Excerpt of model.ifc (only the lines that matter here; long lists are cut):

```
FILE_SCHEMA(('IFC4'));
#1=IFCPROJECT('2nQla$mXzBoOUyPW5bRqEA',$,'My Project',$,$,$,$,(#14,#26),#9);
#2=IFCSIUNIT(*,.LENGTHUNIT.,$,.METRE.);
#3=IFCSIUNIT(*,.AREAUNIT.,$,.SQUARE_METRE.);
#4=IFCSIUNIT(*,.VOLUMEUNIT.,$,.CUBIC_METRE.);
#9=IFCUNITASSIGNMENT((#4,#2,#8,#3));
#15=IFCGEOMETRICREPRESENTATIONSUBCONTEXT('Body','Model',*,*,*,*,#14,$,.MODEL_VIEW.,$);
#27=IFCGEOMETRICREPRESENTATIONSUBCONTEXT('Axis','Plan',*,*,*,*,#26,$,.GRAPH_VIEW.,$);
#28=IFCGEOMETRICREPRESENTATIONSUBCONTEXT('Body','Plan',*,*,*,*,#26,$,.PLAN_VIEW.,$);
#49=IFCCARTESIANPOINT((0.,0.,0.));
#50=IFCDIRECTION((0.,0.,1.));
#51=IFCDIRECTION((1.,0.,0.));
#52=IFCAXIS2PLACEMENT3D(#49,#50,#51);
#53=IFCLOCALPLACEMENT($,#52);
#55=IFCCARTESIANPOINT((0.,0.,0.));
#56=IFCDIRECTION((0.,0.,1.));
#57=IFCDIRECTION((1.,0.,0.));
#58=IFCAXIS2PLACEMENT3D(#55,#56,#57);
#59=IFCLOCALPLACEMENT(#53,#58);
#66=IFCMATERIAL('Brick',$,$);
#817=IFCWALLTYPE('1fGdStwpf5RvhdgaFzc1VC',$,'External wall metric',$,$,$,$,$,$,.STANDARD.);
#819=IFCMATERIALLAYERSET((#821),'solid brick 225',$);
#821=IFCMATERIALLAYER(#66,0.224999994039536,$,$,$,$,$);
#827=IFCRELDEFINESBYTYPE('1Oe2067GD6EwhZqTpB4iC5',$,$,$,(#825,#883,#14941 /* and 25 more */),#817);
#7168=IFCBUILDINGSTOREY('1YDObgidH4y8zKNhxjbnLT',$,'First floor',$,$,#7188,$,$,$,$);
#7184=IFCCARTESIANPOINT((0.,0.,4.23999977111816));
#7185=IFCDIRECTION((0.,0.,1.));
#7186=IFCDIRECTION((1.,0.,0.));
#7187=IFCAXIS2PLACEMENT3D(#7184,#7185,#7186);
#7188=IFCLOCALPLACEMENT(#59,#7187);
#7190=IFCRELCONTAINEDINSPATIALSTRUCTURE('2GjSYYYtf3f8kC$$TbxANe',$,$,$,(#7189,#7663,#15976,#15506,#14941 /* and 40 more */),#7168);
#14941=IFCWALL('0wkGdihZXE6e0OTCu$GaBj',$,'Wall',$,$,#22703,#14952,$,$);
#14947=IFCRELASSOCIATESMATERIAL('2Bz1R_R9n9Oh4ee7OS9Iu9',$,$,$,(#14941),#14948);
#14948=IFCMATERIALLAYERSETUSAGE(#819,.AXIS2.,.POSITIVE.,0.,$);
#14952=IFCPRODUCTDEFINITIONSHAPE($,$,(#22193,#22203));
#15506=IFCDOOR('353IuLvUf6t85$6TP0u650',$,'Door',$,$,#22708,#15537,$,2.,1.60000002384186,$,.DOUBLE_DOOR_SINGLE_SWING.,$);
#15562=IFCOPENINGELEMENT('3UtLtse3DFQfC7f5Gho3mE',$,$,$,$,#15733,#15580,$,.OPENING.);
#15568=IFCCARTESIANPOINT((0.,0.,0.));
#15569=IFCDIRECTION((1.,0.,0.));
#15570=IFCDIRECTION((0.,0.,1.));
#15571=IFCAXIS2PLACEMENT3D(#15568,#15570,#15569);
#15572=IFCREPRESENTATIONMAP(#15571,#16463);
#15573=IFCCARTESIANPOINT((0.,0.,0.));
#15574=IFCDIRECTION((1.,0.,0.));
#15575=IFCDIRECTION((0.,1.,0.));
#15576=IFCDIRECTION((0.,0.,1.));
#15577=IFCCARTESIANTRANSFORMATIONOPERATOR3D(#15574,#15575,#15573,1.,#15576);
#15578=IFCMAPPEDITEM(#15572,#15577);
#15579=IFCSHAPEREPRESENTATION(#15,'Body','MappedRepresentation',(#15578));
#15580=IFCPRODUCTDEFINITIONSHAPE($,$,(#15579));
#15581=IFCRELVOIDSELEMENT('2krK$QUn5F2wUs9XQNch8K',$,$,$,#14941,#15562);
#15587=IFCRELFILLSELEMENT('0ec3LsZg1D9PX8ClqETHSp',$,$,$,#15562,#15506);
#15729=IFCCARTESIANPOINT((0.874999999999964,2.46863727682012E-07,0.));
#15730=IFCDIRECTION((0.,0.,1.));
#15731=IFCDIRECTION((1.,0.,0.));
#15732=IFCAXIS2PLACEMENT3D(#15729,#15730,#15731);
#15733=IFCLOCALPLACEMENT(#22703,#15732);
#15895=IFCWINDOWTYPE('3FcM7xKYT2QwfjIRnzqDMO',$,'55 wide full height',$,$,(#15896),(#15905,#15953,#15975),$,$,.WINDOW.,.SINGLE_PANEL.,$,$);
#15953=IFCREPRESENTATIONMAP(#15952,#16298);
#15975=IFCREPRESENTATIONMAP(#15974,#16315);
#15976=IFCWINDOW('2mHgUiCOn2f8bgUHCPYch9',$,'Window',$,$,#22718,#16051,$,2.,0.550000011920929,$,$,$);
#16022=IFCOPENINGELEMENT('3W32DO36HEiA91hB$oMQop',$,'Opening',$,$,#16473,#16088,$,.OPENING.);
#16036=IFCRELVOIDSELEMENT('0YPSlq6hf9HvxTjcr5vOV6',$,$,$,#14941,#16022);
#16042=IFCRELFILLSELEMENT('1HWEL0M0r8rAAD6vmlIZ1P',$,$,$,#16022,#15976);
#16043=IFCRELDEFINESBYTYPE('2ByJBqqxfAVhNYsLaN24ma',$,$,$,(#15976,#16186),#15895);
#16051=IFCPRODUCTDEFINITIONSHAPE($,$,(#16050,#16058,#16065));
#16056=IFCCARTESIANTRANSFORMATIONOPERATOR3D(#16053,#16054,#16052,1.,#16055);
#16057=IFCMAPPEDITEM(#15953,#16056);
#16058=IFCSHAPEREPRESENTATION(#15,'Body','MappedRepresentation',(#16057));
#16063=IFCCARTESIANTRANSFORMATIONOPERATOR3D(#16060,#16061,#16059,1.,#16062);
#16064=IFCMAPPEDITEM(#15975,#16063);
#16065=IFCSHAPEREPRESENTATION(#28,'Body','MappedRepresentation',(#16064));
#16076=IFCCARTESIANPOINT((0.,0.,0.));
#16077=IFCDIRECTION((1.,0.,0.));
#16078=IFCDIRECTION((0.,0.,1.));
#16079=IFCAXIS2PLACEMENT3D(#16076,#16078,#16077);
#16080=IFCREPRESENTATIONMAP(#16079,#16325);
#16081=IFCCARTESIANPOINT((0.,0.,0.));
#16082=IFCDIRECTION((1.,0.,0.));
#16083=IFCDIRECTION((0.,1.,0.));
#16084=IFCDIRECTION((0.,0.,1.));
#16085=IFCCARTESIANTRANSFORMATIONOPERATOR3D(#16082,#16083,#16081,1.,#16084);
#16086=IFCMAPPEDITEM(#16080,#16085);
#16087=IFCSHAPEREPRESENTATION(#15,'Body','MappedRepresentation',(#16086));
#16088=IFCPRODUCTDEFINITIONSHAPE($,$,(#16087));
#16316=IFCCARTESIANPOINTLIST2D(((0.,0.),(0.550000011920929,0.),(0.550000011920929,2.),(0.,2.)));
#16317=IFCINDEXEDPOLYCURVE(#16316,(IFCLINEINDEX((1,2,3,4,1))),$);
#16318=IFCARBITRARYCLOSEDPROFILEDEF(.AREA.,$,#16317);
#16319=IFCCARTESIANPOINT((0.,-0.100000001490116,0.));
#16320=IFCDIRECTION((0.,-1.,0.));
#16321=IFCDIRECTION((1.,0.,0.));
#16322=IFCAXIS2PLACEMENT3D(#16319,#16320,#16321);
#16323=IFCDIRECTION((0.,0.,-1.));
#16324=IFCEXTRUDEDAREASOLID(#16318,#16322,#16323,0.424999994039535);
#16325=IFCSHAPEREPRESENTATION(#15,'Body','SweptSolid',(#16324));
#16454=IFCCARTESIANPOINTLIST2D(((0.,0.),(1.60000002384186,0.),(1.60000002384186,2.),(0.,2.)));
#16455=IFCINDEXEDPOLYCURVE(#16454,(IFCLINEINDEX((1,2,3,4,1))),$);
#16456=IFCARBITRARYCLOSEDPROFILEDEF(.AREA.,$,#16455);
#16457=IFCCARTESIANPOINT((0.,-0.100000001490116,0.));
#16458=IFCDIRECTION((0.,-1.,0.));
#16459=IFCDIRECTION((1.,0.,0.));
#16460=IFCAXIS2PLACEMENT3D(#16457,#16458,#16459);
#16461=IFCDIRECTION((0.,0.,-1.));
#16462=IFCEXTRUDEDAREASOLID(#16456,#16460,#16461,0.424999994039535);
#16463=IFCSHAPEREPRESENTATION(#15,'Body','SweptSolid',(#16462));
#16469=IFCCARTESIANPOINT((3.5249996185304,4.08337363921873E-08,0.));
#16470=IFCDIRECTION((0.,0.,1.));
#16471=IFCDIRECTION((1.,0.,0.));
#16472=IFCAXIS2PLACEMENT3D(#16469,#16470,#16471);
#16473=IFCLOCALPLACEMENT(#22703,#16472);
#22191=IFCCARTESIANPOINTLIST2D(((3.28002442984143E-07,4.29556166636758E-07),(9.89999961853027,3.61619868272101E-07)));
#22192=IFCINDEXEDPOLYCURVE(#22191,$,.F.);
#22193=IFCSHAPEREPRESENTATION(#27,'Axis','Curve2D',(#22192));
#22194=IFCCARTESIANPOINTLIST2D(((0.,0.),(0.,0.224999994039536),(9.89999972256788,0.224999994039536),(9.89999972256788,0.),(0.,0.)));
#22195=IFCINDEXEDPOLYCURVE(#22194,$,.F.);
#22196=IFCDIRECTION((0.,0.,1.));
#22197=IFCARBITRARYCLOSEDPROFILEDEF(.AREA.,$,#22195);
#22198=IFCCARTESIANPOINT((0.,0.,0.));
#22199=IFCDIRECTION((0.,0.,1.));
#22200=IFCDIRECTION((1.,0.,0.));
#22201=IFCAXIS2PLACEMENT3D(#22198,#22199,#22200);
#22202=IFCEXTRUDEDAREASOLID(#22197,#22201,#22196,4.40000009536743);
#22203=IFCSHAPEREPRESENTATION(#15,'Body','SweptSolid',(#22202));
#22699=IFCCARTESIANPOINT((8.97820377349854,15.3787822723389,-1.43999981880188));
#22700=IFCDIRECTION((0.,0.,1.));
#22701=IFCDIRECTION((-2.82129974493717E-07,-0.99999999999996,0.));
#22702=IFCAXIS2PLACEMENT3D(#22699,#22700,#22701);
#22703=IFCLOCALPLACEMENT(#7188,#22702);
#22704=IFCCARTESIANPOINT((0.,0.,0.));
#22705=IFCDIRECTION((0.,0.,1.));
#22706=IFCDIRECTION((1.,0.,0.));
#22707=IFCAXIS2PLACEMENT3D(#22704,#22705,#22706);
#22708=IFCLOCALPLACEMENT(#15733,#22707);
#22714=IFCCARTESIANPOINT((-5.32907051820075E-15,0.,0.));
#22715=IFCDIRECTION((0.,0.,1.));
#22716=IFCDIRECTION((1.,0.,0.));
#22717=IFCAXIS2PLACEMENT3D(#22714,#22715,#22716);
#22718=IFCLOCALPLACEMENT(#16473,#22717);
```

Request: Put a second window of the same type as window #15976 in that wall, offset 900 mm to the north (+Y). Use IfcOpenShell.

```python
import ifcopenshell
import ifcopenshell.api.feature
import ifcopenshell.api.geometry
import ifcopenshell.api.root
import ifcopenshell.geom
import ifcopenshell.util.element
import ifcopenshell.util.placement
import ifcopenshell.util.shape
import ifcopenshell.util.unit

model = ifcopenshell.open("model.ifc")
unit_scale = ifcopenshell.util.unit.calculate_unit_scale(model)
settings = ifcopenshell.geom.settings()


def volume(element):
    """Net volume in cubic metres, openings subtracted."""
    shape = ifcopenshell.geom.create_shape(settings, element)
    return ifcopenshell.util.shape.get_volume(shape.geometry)


window = model.by_guid("2mHgUiCOn2f8bgUHCPYch9")
opening = window.FillsVoids[0].RelatingOpeningElement
wall = opening.VoidsElements[0].RelatingBuildingElement
before = volume(wall)
shift = ifcopenshell.util.placement.get_local_placement(wall.ObjectPlacement)[:3, 0] * -0.9 / unit_scale

# copy_class copies the void relationship, type, container and properties, but no geometry.
new_opening = ifcopenshell.api.root.copy_class(model, product=opening)
new_opening.Representation = ifcopenshell.util.element.copy_deep(
    model, opening.Representation, exclude=["IfcGeometricRepresentationContext", "IfcRepresentationMap"]
)
new_window = ifcopenshell.api.root.copy_class(model, product=window)
new_window.Representation = ifcopenshell.util.element.copy_deep(
    model, window.Representation, exclude=["IfcGeometricRepresentationContext", "IfcRepresentationMap"]
)
ifcopenshell.api.feature.add_filling(model, opening=new_opening, element=new_window)

for old, new in ((opening, new_opening), (window, new_window)):
    matrix = ifcopenshell.util.placement.get_local_placement(old.ObjectPlacement)
    matrix[:3, 3] += shift
    ifcopenshell.api.geometry.edit_object_placement(model, product=new, matrix=matrix, is_si=False)

after = volume(wall)

print(f"wall volume {before:.3f} -> {after:.3f} m3")

model.write("model-out.ifc")
```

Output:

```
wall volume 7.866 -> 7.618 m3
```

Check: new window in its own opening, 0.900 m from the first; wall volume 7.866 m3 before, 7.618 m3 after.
